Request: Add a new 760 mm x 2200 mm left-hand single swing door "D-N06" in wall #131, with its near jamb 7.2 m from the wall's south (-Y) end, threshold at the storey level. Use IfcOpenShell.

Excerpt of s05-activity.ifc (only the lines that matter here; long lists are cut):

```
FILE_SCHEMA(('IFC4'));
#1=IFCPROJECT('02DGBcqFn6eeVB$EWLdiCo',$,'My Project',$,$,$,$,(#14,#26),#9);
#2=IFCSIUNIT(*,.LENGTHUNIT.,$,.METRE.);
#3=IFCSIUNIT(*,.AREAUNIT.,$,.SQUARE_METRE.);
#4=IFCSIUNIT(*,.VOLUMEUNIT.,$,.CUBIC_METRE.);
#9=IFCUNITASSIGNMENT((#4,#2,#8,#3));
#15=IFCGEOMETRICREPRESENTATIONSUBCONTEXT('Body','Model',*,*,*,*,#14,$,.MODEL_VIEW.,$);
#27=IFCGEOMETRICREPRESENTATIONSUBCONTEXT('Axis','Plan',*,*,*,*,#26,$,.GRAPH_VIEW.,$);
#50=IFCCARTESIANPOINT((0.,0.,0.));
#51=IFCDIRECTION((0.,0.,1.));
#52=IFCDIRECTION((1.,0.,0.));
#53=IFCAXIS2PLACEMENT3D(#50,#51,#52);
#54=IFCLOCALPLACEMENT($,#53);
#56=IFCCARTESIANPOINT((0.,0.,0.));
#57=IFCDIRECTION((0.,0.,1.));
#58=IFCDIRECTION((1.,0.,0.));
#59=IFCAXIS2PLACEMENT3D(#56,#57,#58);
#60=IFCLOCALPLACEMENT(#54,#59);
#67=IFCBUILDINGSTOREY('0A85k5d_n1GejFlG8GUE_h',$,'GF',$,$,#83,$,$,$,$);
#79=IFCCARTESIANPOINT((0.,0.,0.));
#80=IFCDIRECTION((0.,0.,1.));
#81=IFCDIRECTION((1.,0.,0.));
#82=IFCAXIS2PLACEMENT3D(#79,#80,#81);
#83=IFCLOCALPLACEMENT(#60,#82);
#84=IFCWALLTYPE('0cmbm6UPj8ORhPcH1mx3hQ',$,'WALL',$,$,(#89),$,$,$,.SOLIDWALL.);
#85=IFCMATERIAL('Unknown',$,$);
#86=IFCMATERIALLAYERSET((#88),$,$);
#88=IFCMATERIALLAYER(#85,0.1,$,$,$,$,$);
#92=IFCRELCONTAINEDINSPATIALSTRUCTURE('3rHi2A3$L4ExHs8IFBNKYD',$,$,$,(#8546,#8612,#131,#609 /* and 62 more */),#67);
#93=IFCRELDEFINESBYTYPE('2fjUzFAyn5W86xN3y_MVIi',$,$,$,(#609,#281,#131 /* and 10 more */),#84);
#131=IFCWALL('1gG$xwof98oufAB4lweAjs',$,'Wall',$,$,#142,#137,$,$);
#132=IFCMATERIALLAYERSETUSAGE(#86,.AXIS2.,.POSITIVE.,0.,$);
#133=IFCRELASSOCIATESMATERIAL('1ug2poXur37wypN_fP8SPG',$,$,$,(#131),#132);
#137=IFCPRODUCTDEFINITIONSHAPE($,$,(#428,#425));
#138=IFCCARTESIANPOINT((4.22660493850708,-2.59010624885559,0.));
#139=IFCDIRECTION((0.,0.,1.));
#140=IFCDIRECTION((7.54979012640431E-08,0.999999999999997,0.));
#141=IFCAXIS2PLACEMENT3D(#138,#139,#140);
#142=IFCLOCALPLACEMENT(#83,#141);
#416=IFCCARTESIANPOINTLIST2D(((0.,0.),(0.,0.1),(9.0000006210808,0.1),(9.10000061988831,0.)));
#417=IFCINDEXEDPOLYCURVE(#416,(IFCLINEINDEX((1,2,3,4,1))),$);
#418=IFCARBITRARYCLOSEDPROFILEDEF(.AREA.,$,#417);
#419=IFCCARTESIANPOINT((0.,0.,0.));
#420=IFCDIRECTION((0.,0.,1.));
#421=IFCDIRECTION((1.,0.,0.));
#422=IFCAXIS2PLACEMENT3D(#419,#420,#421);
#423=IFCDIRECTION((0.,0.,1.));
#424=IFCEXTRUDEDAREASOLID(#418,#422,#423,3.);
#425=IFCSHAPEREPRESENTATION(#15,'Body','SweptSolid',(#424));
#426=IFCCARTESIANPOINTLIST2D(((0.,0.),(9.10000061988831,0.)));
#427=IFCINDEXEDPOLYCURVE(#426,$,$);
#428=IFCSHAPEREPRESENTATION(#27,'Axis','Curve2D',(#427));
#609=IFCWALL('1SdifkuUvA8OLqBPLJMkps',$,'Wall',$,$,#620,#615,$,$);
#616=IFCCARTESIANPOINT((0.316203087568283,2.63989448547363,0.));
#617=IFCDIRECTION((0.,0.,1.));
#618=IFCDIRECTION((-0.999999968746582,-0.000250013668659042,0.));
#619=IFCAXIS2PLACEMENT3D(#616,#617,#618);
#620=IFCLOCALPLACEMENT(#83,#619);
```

```python
import numpy as np
import ifcopenshell
import ifcopenshell.api.feature
import ifcopenshell.api.geometry
import ifcopenshell.api.root
import ifcopenshell.api.spatial
import ifcopenshell.geom
import ifcopenshell.util.element
import ifcopenshell.util.placement
import ifcopenshell.util.representation
import ifcopenshell.util.shape
import ifcopenshell.util.unit

model = ifcopenshell.open("s05-activity.ifc")
unit_scale = ifcopenshell.util.unit.calculate_unit_scale(model)
settings = ifcopenshell.geom.settings()


def volume(element):
    """Net volume in cubic metres, openings subtracted."""
    shape = ifcopenshell.geom.create_shape(settings, element)
    return ifcopenshell.util.shape.get_volume(shape.geometry)


wall = model.by_guid("1gG$xwof98oufAB4lweAjs")
storey = ifcopenshell.util.element.get_container(wall, ifc_class="IfcBuildingStorey")
context = ifcopenshell.util.representation.get_context(model, "Model", "Body", "MODEL_VIEW")
before = volume(wall)

width, height, from_end, sill = 0.76, 2.2, 7.2, 0.0  # metres

# The wall runs along its own X axis, and the end named is its -X end.
wall_shape = ifcopenshell.geom.create_shape(settings, wall)
x, y, z = ifcopenshell.util.shape.get_vertices(wall_shape.geometry).T
start = x.min() + from_end
face, thickness = float(y.min()), float(y.max() - y.min())
wall_matrix = ifcopenshell.util.placement.get_local_placement(wall.ObjectPlacement)
level = ifcopenshell.util.placement.get_local_placement(storey.ObjectPlacement)[2, 3]


def in_wall(x, y):
    """Placement at x, y metres in the wall's axes, at sill height."""
    matrix = wall_matrix.copy()
    matrix[:, 3] = wall_matrix @ np.array([x / unit_scale, y / unit_scale, 0.0, 1.0])
    matrix[2, 3] = level + sill / unit_scale
    return matrix


# Opening: a box that overshoots both wall faces by 50 mm.
opening = ifcopenshell.api.root.create_entity(model, ifc_class="IfcOpeningElement", predefined_type="OPENING")
box = ifcopenshell.api.geometry.add_wall_representation(
    model, context=context, length=width, height=height, thickness=thickness + 0.1
)
ifcopenshell.api.geometry.assign_representation(model, product=opening, representation=box)
ifcopenshell.api.geometry.edit_object_placement(model, product=opening, matrix=in_wall(start, face - 0.05), is_si=False)
ifcopenshell.api.feature.add_feature(model, feature=opening, element=wall)

door = ifcopenshell.api.root.create_entity(model, ifc_class="IfcDoor", name="D-N06", predefined_type="DOOR")
door.OverallWidth, door.OverallHeight = width / unit_scale, height / unit_scale
door.OperationType = "SINGLE_SWING_LEFT"
body = ifcopenshell.api.geometry.add_door_representation(
    model,
    context=context,
    overall_width=door.OverallWidth,
    overall_height=door.OverallHeight,
    operation_type="SINGLE_SWING_LEFT",
    lining_properties={"LiningDepth": thickness / unit_scale, "ThresholdDepth": thickness / unit_scale},
)
ifcopenshell.api.geometry.assign_representation(model, product=door, representation=body)
ifcopenshell.api.spatial.assign_container(model, products=[door], relating_structure=storey)
ifcopenshell.api.feature.add_filling(model, opening=opening, element=door)

# The lining spans the wall, so the door starts at the wall face.
ifcopenshell.api.geometry.edit_object_placement(model, product=door, matrix=in_wall(start, face), is_si=False)

after = volume(wall)

print(f"wall volume {before:.3f} -> {after:.3f} m3")

model.write("s05-activity_rev.ifc")
```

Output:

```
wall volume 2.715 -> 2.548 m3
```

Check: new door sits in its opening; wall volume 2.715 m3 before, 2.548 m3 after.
